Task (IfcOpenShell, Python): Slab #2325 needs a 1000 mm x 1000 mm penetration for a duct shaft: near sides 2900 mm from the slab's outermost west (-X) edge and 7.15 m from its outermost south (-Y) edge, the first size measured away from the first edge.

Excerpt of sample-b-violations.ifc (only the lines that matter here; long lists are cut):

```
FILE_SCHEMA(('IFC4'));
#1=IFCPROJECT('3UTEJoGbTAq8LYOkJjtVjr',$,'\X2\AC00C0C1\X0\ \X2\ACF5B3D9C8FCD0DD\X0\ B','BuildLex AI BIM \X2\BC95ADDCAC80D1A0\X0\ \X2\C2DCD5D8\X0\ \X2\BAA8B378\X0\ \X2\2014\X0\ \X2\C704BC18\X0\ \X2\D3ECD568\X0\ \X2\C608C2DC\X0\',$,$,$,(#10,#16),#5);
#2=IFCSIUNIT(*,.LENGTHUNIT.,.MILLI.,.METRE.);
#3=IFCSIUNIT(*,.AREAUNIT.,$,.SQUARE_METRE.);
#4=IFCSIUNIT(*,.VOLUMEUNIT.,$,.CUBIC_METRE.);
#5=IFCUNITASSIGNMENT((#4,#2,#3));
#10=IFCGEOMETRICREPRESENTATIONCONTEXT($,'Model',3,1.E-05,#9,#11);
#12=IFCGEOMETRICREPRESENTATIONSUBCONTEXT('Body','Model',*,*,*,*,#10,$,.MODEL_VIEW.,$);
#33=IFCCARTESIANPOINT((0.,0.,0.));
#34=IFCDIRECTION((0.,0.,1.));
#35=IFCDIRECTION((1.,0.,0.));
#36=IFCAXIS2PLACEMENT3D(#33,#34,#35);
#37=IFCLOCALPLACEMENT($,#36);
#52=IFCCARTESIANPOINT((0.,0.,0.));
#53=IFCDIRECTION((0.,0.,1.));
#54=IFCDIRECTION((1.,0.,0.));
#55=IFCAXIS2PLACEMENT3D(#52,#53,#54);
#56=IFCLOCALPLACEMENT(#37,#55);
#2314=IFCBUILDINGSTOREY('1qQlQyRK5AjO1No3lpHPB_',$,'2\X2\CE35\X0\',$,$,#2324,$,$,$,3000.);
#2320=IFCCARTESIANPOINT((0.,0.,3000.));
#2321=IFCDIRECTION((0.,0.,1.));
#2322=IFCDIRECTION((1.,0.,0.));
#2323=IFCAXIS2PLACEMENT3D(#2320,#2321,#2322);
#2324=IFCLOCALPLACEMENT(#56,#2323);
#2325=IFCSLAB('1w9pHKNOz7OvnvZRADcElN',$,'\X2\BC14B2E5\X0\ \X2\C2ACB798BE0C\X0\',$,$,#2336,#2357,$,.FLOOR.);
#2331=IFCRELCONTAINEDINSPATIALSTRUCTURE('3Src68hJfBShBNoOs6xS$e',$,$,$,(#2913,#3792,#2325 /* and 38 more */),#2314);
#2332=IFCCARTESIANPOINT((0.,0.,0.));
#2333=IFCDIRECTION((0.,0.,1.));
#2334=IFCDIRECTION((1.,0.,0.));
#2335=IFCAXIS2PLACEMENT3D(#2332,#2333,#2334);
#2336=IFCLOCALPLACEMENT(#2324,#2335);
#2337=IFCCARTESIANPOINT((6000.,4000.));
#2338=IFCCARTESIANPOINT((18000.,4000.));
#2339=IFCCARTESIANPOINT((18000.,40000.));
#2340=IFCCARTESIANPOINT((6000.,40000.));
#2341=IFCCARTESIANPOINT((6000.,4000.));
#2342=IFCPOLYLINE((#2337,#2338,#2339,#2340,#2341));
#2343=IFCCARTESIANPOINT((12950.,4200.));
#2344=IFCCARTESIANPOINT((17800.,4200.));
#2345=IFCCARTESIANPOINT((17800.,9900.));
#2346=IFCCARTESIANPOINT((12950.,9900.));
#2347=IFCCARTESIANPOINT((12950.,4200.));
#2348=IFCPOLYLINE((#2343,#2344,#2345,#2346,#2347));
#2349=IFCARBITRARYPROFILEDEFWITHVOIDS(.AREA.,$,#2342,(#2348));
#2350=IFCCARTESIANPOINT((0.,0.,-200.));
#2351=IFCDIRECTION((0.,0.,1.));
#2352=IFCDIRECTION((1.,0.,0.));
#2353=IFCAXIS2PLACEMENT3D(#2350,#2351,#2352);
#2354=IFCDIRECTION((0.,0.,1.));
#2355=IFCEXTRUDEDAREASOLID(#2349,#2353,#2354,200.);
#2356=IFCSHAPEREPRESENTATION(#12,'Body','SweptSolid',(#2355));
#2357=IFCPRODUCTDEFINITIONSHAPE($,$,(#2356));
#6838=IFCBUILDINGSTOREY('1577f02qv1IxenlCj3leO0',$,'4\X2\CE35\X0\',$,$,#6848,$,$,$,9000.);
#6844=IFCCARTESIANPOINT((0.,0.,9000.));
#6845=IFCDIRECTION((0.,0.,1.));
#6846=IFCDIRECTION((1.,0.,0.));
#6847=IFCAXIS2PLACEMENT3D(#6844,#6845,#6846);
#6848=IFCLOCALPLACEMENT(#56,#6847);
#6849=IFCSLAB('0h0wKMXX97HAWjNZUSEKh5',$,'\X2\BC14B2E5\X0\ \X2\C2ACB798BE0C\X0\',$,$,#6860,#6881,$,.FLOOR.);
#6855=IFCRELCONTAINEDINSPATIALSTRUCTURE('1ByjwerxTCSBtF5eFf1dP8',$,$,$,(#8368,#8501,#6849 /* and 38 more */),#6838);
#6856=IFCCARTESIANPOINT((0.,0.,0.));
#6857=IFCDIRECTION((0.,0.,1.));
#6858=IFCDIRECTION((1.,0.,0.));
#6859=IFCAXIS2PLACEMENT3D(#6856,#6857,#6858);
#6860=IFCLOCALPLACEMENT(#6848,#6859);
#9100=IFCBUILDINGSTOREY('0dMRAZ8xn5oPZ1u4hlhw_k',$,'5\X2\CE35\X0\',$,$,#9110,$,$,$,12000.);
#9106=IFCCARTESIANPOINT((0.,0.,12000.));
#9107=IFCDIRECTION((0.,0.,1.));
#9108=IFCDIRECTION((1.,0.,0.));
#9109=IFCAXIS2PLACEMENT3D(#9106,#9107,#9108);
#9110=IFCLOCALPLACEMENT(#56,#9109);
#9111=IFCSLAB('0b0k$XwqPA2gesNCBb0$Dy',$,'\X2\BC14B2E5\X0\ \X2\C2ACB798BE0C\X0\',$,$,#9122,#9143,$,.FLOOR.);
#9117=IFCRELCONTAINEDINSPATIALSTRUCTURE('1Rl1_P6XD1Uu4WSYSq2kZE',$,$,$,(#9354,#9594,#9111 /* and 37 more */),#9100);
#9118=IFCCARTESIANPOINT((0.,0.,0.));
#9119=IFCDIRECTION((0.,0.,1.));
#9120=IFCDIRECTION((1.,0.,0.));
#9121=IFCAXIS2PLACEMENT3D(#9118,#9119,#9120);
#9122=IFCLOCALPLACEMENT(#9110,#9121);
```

```python
import numpy as np
import ifcopenshell
import ifcopenshell.api.feature
import ifcopenshell.api.geometry
import ifcopenshell.api.root
import ifcopenshell.geom
import ifcopenshell.util.placement
import ifcopenshell.util.representation
import ifcopenshell.util.shape
import ifcopenshell.util.unit

model = ifcopenshell.open("sample-b-violations.ifc")
unit_scale = ifcopenshell.util.unit.calculate_unit_scale(model)
settings = ifcopenshell.geom.settings()


def volume(element):
    """Net volume in cubic metres, openings subtracted."""
    shape = ifcopenshell.geom.create_shape(settings, element)
    return ifcopenshell.util.shape.get_volume(shape.geometry)


slab = model.by_guid("1w9pHKNOz7OvnvZRADcElN")
before = volume(slab)

# Extent in the slab's own axes, in metres. The edges named are its -X and -Y sides.
slab_shape = ifcopenshell.geom.create_shape(settings, slab)
vertices = ifcopenshell.util.shape.get_vertices(slab_shape.geometry)
x_min, y_min, bottom = vertices.min(axis=0)
top = vertices[:, 2].max()

opening = ifcopenshell.api.root.create_entity(model, ifc_class="IfcOpeningElement", name="Duct shaft opening", predefined_type="OPENING")
context = ifcopenshell.util.representation.get_context(model, "Model", "Body", "MODEL_VIEW")
width, depth = 1, 1
outline = [(0.0, 0.0), (width, 0.0), (width, depth), (0.0, depth), (0.0, 0.0)]
# Overshoot both faces by 50 mm so the cut is clean.
shape = ifcopenshell.api.geometry.add_slab_representation(
    model, context=context, depth=top - bottom + 0.1, polyline=outline
)
ifcopenshell.api.geometry.assign_representation(model, product=opening, representation=shape)

matrix = ifcopenshell.util.placement.get_local_placement(slab.ObjectPlacement)
matrix[:, 3] = matrix @ np.append(np.array([x_min + 2.9, y_min + 7.15, bottom - 0.05]) / unit_scale, 1.0)
ifcopenshell.api.geometry.edit_object_placement(model, product=opening, matrix=matrix, is_si=False)
ifcopenshell.api.feature.add_feature(model, feature=opening, element=slab)

after = volume(slab)

print(f"slab volume {before:.3f} -> {after:.3f} m3")

model.write("sample-b-violations_edited.ifc")
```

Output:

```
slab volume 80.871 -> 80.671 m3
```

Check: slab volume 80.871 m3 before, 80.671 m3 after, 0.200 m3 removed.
